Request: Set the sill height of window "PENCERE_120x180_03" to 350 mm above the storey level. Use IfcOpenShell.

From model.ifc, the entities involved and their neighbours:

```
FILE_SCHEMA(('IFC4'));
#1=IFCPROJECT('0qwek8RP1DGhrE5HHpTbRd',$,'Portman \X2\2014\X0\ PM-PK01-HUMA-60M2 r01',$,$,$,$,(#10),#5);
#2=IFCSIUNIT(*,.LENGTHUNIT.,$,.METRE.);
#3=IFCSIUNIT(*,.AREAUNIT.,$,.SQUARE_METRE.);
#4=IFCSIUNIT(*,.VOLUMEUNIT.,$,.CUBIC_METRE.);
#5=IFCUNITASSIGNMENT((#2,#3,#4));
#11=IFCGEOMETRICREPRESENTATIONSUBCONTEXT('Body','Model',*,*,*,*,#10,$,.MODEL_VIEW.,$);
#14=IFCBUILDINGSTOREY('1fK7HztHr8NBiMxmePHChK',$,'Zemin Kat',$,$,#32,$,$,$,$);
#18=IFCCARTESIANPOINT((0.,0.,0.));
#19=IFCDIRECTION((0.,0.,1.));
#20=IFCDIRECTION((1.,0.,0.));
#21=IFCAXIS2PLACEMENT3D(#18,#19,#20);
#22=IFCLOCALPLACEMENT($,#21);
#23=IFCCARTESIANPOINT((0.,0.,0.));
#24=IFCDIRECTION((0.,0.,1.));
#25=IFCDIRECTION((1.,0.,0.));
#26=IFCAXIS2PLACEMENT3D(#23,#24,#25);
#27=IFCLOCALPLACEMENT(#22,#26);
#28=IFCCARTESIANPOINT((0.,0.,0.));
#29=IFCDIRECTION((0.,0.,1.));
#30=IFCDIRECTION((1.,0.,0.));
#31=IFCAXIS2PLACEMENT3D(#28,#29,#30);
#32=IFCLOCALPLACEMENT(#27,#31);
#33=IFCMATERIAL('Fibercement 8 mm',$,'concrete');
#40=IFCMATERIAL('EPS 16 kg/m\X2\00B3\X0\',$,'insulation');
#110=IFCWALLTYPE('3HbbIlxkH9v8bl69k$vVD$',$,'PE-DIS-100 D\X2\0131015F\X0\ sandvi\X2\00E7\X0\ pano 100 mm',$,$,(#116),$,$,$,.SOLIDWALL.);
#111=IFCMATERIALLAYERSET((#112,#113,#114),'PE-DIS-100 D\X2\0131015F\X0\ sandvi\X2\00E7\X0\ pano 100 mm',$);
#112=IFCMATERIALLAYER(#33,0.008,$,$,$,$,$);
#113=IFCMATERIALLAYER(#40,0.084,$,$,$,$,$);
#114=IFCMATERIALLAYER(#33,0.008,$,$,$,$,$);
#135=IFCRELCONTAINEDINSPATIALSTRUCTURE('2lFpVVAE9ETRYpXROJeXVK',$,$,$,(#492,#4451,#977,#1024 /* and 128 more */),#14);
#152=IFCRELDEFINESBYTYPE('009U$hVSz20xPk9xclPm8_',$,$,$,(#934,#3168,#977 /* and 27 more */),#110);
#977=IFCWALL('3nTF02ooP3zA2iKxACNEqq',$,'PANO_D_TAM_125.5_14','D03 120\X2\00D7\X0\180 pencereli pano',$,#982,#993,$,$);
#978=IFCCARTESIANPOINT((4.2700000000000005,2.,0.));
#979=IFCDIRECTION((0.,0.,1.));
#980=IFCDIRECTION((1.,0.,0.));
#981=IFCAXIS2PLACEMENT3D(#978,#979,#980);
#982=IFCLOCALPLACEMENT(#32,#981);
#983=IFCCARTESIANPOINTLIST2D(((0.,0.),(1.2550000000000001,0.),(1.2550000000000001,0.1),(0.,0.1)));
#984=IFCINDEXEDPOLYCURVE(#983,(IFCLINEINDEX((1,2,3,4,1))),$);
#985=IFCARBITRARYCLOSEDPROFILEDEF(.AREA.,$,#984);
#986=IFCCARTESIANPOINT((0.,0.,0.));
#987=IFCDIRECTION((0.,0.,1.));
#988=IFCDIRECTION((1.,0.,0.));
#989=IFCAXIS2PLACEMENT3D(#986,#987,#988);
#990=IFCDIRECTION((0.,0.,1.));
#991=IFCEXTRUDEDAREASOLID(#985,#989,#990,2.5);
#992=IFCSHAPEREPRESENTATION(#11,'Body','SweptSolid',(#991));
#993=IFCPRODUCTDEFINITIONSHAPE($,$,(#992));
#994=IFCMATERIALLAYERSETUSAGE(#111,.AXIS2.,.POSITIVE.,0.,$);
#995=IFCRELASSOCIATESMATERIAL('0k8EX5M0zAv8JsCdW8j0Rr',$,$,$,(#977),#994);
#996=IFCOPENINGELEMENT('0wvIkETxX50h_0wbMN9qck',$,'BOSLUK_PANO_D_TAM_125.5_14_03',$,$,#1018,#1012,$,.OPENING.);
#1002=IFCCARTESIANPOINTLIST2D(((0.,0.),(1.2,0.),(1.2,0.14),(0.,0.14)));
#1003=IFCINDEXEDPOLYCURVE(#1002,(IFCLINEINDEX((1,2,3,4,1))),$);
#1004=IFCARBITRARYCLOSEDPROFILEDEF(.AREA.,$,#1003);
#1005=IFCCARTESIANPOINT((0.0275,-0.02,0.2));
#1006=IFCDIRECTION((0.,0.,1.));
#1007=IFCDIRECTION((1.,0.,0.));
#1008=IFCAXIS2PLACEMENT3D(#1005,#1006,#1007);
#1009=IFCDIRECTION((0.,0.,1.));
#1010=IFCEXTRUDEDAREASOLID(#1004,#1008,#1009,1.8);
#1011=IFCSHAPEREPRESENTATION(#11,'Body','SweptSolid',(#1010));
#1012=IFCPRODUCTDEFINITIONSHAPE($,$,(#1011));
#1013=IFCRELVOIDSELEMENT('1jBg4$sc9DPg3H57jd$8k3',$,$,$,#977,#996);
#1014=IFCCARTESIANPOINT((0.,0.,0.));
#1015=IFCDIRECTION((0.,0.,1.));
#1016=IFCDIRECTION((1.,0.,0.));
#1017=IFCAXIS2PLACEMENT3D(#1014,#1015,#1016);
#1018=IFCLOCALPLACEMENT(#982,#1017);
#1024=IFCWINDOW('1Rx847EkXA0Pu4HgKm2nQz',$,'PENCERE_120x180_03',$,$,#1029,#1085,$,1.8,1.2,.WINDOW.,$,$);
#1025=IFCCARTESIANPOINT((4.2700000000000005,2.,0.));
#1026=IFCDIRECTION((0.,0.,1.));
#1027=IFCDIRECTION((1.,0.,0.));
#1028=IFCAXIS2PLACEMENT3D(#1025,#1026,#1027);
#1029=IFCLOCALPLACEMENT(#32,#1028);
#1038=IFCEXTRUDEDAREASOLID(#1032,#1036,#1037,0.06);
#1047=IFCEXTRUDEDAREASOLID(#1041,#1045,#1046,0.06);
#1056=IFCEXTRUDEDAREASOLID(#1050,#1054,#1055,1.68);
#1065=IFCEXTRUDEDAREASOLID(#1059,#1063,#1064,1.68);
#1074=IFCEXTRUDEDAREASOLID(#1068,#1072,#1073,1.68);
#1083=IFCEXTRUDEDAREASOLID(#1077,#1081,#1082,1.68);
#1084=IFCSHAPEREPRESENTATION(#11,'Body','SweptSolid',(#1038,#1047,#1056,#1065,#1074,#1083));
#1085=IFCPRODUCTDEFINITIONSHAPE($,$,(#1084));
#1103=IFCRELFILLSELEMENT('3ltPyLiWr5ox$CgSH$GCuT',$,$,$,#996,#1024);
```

```python
import numpy as np
import ifcopenshell
import ifcopenshell.api.geometry
import ifcopenshell.geom
import ifcopenshell.util.element
import ifcopenshell.util.placement
import ifcopenshell.util.shape
import ifcopenshell.util.unit

model = ifcopenshell.open("model.ifc")
unit_scale = ifcopenshell.util.unit.calculate_unit_scale(model)

window = model.by_guid("1Rx847EkXA0Pu4HgKm2nQz")
opening = window.FillsVoids[0].RelatingOpeningElement
storey = ifcopenshell.util.element.get_container(window, ifc_class="IfcBuildingStorey")
level = ifcopenshell.util.placement.get_local_placement(storey.ObjectPlacement)[2, 3]

# The opening's origin need not be at the sill, so measure its lowest point.
shape = ifcopenshell.geom.create_shape(ifcopenshell.geom.settings(), opening)
bottom = ifcopenshell.util.shape.get_shape_bottom_elevation(shape, shape.geometry) / unit_scale
dz = level + 0.35 - bottom

shift = np.array([0.0, 0.0, dz])
# The window is not placed relative to its opening, so move both.
for product in (opening, window):
    matrix = ifcopenshell.util.placement.get_local_placement(product.ObjectPlacement)
    matrix[:3, 3] += shift
    ifcopenshell.api.geometry.edit_object_placement(model, product=product, matrix=matrix, is_si=False)

print(f"moved by {dz * unit_scale:+.3f} m")

model.write("model_rev.ifc")
```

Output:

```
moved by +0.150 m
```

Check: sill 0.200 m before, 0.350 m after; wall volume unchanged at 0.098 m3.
